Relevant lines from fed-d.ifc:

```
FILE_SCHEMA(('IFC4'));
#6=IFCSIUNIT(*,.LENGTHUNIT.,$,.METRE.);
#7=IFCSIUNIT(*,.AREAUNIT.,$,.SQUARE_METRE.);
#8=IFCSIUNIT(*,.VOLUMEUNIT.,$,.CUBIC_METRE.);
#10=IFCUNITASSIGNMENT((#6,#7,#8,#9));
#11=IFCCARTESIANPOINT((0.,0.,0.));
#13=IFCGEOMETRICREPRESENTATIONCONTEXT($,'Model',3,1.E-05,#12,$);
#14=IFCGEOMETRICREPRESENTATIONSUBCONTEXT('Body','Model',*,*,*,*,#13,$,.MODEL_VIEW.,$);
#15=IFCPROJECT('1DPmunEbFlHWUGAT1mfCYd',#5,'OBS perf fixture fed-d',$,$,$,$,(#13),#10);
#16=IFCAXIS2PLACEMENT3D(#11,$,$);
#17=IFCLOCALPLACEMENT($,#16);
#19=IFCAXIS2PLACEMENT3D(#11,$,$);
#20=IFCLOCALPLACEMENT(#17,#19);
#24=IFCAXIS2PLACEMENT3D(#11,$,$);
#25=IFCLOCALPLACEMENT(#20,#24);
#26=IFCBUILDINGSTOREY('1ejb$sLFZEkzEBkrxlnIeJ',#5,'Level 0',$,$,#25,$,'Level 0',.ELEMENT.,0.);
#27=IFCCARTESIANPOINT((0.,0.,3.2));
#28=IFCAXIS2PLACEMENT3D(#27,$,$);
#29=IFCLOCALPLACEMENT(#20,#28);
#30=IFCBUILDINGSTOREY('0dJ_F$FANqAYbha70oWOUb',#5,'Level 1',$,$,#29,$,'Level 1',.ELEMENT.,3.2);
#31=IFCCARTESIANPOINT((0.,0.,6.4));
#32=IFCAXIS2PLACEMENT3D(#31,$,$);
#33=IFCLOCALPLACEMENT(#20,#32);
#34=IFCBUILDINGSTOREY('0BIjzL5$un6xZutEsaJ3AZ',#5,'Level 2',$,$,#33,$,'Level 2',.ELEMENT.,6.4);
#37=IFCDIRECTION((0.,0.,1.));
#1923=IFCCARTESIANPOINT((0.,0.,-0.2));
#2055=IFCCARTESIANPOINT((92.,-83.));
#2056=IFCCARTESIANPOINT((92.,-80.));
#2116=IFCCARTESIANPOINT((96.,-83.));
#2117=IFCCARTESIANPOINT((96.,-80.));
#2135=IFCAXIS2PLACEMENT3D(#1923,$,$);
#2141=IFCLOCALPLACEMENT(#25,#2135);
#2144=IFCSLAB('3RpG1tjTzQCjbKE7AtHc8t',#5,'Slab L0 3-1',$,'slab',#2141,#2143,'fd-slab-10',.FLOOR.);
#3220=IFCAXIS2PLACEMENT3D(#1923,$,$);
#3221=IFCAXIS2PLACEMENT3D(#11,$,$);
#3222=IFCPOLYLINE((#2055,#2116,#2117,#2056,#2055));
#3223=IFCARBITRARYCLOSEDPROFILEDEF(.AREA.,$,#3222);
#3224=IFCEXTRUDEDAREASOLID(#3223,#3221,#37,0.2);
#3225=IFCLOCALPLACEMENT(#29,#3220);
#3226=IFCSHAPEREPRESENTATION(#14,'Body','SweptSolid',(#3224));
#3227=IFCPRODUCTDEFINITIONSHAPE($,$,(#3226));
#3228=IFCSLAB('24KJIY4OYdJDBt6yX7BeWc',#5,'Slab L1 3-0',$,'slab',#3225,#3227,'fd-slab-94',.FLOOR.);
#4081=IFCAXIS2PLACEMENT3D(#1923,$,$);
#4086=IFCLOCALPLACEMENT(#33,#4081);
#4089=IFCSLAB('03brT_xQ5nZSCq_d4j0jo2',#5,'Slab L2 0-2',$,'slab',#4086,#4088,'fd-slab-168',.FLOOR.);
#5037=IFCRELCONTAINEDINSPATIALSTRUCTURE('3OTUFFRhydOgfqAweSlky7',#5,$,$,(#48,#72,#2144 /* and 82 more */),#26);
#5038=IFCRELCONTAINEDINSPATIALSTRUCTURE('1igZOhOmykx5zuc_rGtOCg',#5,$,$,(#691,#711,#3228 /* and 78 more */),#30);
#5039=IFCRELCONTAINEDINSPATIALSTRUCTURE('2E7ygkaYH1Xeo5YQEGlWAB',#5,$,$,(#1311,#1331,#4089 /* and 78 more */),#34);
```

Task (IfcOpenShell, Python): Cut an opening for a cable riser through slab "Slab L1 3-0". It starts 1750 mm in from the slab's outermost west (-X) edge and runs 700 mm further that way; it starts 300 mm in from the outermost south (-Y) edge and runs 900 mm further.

```python
import numpy as np
import ifcopenshell
import ifcopenshell.api.feature
import ifcopenshell.api.geometry
import ifcopenshell.api.root
import ifcopenshell.geom
import ifcopenshell.util.placement
import ifcopenshell.util.representation
import ifcopenshell.util.shape
import ifcopenshell.util.unit

model = ifcopenshell.open("fed-d.ifc")
unit_scale = ifcopenshell.util.unit.calculate_unit_scale(model)
settings = ifcopenshell.geom.settings()


def volume(element):
    """Net volume in cubic metres, openings subtracted."""
    shape = ifcopenshell.geom.create_shape(settings, element)
    return ifcopenshell.util.shape.get_volume(shape.geometry)


slab = model.by_guid("24KJIY4OYdJDBt6yX7BeWc")
before = volume(slab)

# Extent in the slab's own axes, in metres. The edges named are its -X and -Y sides.
slab_shape = ifcopenshell.geom.create_shape(settings, slab)
vertices = ifcopenshell.util.shape.get_vertices(slab_shape.geometry)
x_min, y_min, bottom = vertices.min(axis=0)
top = vertices[:, 2].max()

opening = ifcopenshell.api.root.create_entity(model, ifc_class="IfcOpeningElement", name="Cable riser opening", predefined_type="OPENING")
context = ifcopenshell.util.representation.get_context(model, "Model", "Body", "MODEL_VIEW")
width, depth = 0.7, 0.9
outline = [(0.0, 0.0), (width, 0.0), (width, depth), (0.0, depth), (0.0, 0.0)]
# Overshoot both faces by 50 mm so the cut is clean.
shape = ifcopenshell.api.geometry.add_slab_representation(
    model, context=context, depth=top - bottom + 0.1, polyline=outline
)
ifcopenshell.api.geometry.assign_representation(model, product=opening, representation=shape)

matrix = ifcopenshell.util.placement.get_local_placement(slab.ObjectPlacement)
matrix[:, 3] = matrix @ np.append(np.array([x_min + 1.75, y_min + 0.3, bottom - 0.05]) / unit_scale, 1.0)
ifcopenshell.api.geometry.edit_object_placement(model, product=opening, matrix=matrix, is_si=False)
ifcopenshell.api.feature.add_feature(model, feature=opening, element=slab)

after = volume(slab)

print(f"slab volume {before:.3f} -> {after:.3f} m3")

model.write("fed-d_v2.ifc")
```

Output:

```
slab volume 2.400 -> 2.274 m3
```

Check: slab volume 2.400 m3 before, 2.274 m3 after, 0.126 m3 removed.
